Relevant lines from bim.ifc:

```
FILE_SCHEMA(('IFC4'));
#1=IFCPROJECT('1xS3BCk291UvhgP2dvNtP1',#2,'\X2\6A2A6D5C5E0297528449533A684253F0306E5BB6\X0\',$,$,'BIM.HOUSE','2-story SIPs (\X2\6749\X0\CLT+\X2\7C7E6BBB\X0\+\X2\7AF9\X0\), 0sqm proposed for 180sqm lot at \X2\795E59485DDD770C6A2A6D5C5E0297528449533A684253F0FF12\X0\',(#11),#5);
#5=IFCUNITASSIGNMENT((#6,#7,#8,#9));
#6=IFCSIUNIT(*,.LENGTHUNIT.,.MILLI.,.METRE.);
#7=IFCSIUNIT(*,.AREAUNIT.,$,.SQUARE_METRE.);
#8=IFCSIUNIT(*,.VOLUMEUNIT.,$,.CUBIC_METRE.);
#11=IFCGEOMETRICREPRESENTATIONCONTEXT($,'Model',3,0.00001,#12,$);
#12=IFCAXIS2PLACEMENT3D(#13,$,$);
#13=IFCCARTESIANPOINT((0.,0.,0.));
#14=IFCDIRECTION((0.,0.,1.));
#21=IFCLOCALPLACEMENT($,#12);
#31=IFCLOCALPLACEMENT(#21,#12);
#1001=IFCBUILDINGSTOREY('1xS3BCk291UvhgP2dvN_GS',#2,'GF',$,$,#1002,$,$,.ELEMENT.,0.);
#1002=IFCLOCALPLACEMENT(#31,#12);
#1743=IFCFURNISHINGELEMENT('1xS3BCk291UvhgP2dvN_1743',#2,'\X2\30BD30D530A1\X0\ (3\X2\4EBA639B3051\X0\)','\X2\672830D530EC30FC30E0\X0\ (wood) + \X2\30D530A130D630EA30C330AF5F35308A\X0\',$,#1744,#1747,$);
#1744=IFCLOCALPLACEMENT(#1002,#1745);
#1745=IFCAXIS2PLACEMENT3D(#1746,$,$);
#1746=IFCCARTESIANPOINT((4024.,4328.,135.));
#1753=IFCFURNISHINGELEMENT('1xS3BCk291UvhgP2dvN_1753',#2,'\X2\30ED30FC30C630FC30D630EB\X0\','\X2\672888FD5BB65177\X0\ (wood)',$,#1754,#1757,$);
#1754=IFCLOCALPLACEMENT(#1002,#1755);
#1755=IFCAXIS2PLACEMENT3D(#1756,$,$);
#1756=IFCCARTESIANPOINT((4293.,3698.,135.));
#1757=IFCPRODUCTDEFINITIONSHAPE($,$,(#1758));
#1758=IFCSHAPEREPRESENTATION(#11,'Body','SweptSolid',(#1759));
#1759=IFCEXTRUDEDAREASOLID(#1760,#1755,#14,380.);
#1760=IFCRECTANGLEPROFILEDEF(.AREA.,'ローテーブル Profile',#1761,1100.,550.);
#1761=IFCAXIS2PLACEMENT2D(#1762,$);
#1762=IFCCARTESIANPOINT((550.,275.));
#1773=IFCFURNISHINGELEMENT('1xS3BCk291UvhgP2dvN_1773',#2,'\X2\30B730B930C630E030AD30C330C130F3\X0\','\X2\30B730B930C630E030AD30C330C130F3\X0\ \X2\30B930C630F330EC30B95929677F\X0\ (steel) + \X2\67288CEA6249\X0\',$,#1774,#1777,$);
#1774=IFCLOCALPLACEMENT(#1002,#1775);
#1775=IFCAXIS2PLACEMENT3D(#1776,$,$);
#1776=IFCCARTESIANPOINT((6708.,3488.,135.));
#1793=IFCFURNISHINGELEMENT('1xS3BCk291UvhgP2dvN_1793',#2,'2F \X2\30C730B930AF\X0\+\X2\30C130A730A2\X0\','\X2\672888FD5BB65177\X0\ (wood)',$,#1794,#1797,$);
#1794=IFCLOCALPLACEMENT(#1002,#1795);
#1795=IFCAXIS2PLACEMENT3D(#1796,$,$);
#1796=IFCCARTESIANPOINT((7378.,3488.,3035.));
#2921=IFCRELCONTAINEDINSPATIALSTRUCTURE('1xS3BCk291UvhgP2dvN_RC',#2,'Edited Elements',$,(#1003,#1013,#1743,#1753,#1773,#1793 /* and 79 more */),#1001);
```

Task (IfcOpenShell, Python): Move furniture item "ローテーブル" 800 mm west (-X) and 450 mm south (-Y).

```python
import ifcopenshell
import ifcopenshell.api.geometry
import ifcopenshell.util.placement

model = ifcopenshell.open("bim.ifc")

item = model.by_guid("1xS3BCk291UvhgP2dvN_1753")
matrix = ifcopenshell.util.placement.get_local_placement(item.ObjectPlacement)
matrix[0, 3] -= 800.0
matrix[1, 3] -= 450.0
ifcopenshell.api.geometry.edit_object_placement(model, product=item, matrix=matrix, is_si=False)

print(ifcopenshell.util.placement.get_local_placement(item.ObjectPlacement).round(3) + 0.0)

model.write("bim_rev.ifc")
```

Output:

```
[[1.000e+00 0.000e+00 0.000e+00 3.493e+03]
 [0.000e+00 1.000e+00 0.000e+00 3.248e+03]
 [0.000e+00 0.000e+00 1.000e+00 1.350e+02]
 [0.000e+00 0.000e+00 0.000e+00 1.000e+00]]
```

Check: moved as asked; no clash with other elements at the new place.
